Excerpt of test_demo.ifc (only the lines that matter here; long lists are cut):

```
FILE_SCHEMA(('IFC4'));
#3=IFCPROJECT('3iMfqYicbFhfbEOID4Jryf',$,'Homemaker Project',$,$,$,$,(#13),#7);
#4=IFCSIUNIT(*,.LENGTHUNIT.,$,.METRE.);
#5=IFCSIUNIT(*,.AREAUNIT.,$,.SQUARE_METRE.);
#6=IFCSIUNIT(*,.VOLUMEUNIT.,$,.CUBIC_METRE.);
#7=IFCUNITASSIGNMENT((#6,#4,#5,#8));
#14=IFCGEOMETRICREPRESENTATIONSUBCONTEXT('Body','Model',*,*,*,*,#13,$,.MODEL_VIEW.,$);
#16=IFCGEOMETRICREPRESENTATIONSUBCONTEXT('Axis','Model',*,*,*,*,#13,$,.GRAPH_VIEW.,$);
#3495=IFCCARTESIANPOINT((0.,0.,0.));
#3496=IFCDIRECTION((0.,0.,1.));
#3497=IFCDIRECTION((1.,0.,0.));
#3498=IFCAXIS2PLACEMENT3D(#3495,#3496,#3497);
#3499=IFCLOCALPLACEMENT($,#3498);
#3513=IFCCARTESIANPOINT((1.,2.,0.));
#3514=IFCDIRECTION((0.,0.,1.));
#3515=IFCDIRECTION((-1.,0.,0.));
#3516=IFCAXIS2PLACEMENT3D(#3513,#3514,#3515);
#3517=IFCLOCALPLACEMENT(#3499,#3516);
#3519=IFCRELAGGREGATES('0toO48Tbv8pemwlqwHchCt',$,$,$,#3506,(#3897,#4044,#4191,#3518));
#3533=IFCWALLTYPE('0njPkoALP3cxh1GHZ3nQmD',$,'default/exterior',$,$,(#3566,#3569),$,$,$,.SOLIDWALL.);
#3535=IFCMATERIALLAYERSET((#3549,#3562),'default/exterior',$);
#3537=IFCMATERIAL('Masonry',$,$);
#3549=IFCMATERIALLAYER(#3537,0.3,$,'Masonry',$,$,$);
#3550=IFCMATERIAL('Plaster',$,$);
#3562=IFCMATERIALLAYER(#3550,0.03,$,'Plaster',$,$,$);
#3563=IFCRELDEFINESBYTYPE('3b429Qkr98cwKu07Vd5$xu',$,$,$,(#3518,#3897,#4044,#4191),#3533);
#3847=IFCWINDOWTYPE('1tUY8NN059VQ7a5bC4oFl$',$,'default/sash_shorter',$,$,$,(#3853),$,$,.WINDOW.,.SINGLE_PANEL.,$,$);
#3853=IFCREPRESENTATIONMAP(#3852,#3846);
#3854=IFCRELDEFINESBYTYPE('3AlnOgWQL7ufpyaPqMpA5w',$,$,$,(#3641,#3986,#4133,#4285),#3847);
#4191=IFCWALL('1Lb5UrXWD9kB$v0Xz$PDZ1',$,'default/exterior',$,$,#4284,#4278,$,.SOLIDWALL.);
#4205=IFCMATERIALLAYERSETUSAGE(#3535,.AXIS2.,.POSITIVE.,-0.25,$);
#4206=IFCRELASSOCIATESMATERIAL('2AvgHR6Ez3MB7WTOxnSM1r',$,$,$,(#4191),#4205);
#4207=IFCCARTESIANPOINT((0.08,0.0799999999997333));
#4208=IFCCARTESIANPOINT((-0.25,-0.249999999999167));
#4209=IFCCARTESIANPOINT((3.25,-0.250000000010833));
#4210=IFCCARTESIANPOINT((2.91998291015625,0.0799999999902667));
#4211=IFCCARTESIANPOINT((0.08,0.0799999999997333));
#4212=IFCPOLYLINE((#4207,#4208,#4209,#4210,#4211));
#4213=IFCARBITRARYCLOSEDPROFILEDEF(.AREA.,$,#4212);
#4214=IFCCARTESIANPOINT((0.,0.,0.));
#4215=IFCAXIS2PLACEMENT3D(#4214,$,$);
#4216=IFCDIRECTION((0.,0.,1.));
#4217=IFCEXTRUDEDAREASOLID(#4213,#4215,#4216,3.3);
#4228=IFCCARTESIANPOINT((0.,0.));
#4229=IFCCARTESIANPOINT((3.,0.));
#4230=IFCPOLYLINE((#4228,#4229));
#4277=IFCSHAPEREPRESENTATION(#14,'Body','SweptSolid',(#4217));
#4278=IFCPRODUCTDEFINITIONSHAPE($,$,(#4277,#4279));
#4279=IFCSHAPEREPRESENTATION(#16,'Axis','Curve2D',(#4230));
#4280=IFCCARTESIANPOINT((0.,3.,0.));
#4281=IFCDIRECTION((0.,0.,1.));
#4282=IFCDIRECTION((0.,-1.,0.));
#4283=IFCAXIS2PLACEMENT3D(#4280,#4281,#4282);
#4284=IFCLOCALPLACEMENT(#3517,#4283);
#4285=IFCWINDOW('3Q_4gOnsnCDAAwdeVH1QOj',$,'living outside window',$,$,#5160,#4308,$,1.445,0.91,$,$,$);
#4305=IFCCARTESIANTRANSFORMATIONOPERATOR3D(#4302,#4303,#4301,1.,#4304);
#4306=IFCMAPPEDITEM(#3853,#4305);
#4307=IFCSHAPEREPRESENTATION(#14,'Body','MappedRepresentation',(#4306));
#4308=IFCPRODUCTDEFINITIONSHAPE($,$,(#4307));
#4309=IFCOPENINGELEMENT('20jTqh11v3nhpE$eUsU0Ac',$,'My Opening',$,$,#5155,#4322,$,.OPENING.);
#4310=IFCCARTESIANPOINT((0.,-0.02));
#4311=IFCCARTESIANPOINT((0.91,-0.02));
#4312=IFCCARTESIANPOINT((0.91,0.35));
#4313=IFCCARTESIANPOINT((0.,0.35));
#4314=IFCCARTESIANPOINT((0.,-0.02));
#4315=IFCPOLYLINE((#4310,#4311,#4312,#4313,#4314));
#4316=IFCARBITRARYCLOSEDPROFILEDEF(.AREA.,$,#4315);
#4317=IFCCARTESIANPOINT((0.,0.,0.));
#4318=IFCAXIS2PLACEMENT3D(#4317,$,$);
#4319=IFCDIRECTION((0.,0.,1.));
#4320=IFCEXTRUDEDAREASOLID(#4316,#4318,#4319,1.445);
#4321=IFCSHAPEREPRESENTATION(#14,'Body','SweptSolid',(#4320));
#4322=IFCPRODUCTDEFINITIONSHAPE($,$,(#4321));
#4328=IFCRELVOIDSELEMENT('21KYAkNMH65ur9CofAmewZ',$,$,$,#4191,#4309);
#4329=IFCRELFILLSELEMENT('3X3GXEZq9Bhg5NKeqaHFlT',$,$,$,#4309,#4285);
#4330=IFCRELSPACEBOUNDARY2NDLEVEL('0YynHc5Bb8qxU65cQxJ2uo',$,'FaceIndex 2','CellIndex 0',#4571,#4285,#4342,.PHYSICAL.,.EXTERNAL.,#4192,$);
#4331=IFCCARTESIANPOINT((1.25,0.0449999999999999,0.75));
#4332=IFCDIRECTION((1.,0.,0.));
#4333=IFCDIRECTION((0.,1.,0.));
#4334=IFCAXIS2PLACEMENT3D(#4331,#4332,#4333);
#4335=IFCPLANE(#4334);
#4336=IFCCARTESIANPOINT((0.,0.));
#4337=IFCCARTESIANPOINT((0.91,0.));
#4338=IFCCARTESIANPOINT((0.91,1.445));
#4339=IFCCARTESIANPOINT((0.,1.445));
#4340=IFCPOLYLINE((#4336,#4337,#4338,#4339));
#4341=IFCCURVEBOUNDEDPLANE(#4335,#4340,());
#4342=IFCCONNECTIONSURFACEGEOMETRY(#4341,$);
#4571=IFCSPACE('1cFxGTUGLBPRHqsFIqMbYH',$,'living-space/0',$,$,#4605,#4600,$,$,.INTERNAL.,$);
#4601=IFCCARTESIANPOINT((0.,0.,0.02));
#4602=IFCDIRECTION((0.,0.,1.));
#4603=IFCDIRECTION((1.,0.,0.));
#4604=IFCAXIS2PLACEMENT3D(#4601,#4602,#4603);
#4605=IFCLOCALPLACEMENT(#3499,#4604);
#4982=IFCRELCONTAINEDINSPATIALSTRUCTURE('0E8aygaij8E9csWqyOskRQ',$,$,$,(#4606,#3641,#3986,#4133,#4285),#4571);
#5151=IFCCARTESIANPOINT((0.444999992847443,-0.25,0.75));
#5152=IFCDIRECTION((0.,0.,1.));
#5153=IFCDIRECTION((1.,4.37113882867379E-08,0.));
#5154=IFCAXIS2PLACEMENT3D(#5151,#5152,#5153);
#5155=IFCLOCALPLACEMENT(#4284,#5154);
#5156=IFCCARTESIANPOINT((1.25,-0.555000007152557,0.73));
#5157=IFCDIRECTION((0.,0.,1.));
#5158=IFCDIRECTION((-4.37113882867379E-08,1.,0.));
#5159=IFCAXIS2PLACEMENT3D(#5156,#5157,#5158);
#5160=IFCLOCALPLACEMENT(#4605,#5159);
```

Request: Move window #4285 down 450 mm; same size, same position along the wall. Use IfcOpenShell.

```python
import numpy as np
import ifcopenshell
import ifcopenshell.api.geometry
import ifcopenshell.util.placement
import ifcopenshell.util.unit

model = ifcopenshell.open("test_demo.ifc")
unit_scale = ifcopenshell.util.unit.calculate_unit_scale(model)

window = model.by_guid("3Q_4gOnsnCDAAwdeVH1QOj")
opening = window.FillsVoids[0].RelatingOpeningElement
dz = -0.45 / unit_scale

shift = np.array([0.0, 0.0, dz])
# The window is not placed relative to its opening, so move both.
for product in (opening, window):
    matrix = ifcopenshell.util.placement.get_local_placement(product.ObjectPlacement)
    matrix[:3, 3] += shift
    ifcopenshell.api.geometry.edit_object_placement(model, product=product, matrix=matrix, is_si=False)

# Space boundary surfaces are stored in each space's coordinates; move them too.
for rel in window.ProvidesBoundaries:
    if not rel.ConnectionGeometry:
        continue
    surface = rel.ConnectionGeometry.SurfaceOnRelatingElement.BasisSurface
    space_matrix = ifcopenshell.util.placement.get_local_placement(rel.RelatingSpace.ObjectPlacement)
    point = np.array(surface.Position.Location.Coordinates) + space_matrix[:3, :3].T @ shift
    surface.Position = model.createIfcAxis2Placement3D(
        model.createIfcCartesianPoint(point.tolist()), surface.Position.Axis, surface.Position.RefDirection
    )

print(f"moved by {dz * unit_scale:+.3f} m")

model.write("test_demo_updated.ifc")
```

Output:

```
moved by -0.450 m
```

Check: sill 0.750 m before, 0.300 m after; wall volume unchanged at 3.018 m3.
